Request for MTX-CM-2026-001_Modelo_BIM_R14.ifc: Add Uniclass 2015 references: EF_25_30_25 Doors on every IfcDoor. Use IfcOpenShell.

First a look at what the model holds.

```python
import ifcopenshell

model = ifcopenshell.open("MTX-CM-2026-001_Modelo_BIM_R14.ifc")
print(model.schema)
print("classifications:", [c.Name for c in model.by_type("IfcClassification")])
for ifc_class in ("IfcDoor", "IfcRoof", "IfcStair", "IfcWall", "IfcWindow"):
    print(ifc_class, len(model.by_type(ifc_class)))
```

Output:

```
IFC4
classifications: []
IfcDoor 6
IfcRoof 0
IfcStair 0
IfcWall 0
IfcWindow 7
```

```python
import ifcopenshell
import ifcopenshell.api.classification

model = ifcopenshell.open("MTX-CM-2026-001_Modelo_BIM_R14.ifc")

system = ifcopenshell.api.classification.add_classification(model, classification="Uniclass 2015")

codes = {
    "IfcDoor": ("EF_25_30_25", "Doors"),
}
for ifc_class, (code, name) in codes.items():
    products = model.by_type(ifc_class)
    ifcopenshell.api.classification.add_reference(
        model, products=products, classification=system, identification=code, name=name
    )
    print(code, len(products))

model.write("MTX-CM-2026-001_Modelo_BIM_R14_updated.ifc")
```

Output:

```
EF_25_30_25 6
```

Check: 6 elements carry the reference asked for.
